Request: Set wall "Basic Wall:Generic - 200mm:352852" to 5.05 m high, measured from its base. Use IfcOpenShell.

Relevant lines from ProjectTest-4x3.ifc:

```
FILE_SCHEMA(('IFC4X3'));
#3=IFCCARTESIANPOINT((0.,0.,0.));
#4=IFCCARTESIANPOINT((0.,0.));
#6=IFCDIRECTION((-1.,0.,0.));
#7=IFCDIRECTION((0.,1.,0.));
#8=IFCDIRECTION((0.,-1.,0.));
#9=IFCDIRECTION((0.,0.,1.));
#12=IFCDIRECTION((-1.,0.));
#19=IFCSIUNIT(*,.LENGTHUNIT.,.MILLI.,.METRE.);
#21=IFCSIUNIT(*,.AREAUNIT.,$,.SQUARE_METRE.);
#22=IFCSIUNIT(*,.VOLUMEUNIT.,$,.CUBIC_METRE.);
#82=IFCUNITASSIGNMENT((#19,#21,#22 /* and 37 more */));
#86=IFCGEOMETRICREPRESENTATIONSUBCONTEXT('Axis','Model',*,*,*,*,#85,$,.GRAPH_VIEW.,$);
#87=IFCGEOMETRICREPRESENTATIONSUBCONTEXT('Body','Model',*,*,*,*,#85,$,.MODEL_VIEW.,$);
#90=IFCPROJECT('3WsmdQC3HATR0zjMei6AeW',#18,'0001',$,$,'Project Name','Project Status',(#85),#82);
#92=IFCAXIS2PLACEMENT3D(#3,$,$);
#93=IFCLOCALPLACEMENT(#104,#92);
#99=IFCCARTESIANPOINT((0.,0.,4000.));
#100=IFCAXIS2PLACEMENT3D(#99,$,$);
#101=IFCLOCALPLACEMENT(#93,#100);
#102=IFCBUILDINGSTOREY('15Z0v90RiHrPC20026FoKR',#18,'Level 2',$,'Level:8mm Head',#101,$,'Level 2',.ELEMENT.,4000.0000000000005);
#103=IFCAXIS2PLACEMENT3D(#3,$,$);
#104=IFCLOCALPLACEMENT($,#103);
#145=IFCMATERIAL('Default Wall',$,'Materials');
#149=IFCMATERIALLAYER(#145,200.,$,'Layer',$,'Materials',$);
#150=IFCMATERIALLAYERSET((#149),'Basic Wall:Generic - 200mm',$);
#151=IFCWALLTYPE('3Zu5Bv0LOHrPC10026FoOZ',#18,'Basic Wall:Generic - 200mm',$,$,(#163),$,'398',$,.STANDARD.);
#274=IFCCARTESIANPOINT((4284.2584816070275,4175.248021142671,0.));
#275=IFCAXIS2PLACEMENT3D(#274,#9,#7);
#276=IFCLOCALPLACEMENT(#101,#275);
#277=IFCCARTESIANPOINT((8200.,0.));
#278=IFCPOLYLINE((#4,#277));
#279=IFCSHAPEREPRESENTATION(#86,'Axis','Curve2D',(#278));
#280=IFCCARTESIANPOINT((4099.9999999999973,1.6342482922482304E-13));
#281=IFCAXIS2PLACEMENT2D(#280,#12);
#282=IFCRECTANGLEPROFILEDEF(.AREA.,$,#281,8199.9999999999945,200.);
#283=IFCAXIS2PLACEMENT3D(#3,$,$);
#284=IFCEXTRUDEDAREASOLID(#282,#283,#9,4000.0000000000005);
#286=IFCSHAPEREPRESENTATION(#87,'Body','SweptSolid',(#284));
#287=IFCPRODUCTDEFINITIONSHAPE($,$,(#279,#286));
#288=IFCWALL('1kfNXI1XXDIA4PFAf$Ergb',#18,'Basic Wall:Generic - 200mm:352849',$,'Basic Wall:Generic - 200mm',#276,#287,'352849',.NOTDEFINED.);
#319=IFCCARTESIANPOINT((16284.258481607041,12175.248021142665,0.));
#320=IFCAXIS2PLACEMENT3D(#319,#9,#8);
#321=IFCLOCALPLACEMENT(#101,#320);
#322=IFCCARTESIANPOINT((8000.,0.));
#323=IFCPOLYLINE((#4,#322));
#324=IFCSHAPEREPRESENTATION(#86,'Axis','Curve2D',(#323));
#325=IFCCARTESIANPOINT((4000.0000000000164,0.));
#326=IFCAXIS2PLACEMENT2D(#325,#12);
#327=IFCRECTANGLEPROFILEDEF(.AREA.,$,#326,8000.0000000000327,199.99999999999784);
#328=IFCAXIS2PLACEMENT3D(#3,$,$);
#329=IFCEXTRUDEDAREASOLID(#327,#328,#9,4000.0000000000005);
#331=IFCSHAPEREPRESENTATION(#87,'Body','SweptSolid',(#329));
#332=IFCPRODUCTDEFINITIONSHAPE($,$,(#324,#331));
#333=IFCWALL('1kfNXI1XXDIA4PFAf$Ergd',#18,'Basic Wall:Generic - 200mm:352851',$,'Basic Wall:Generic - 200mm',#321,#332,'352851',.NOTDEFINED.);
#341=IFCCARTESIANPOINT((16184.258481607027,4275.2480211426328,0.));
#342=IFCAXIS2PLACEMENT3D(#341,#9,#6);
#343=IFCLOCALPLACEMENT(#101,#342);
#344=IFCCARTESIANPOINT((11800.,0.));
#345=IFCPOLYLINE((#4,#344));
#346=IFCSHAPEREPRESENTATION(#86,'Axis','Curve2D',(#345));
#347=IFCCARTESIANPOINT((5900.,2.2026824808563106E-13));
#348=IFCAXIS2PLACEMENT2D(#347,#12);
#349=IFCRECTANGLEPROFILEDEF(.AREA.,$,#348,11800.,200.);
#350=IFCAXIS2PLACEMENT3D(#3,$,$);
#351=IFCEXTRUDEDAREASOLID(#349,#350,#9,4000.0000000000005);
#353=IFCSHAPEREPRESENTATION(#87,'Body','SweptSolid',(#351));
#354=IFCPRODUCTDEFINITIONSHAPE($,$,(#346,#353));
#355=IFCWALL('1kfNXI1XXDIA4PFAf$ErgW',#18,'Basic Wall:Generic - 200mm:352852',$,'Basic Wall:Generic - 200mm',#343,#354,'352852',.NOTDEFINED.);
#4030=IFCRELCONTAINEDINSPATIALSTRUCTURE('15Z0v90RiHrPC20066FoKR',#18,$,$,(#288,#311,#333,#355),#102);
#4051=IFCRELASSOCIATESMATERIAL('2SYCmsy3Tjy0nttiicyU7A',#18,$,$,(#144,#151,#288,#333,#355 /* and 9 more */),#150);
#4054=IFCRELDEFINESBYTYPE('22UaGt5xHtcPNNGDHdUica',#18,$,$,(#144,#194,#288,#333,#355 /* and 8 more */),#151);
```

```python
import ifcopenshell
import ifcopenshell.geom
import ifcopenshell.util.representation
import ifcopenshell.util.shape

model = ifcopenshell.open("ProjectTest-4x3.ifc")
settings = ifcopenshell.geom.settings()


def volume(element):
    """Net volume in cubic metres, openings subtracted."""
    shape = ifcopenshell.geom.create_shape(settings, element)
    return ifcopenshell.util.shape.get_volume(shape.geometry)


wall = model.by_guid("1kfNXI1XXDIA4PFAf$ErgW")
before = volume(wall)

body = ifcopenshell.util.representation.get_representation(wall, "Model", "Body")
solid = body.Items[0]
old_height = solid.Depth
solid.Depth = 5050.0
after = volume(wall)

print(f"height {old_height:g} -> {solid.Depth:g}, volume {before:.3f} -> {after:.3f} m3")

model.write("ProjectTest-4x3_edited.ifc")
```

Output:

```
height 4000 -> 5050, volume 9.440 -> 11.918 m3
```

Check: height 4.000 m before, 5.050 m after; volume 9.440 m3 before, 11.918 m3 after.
